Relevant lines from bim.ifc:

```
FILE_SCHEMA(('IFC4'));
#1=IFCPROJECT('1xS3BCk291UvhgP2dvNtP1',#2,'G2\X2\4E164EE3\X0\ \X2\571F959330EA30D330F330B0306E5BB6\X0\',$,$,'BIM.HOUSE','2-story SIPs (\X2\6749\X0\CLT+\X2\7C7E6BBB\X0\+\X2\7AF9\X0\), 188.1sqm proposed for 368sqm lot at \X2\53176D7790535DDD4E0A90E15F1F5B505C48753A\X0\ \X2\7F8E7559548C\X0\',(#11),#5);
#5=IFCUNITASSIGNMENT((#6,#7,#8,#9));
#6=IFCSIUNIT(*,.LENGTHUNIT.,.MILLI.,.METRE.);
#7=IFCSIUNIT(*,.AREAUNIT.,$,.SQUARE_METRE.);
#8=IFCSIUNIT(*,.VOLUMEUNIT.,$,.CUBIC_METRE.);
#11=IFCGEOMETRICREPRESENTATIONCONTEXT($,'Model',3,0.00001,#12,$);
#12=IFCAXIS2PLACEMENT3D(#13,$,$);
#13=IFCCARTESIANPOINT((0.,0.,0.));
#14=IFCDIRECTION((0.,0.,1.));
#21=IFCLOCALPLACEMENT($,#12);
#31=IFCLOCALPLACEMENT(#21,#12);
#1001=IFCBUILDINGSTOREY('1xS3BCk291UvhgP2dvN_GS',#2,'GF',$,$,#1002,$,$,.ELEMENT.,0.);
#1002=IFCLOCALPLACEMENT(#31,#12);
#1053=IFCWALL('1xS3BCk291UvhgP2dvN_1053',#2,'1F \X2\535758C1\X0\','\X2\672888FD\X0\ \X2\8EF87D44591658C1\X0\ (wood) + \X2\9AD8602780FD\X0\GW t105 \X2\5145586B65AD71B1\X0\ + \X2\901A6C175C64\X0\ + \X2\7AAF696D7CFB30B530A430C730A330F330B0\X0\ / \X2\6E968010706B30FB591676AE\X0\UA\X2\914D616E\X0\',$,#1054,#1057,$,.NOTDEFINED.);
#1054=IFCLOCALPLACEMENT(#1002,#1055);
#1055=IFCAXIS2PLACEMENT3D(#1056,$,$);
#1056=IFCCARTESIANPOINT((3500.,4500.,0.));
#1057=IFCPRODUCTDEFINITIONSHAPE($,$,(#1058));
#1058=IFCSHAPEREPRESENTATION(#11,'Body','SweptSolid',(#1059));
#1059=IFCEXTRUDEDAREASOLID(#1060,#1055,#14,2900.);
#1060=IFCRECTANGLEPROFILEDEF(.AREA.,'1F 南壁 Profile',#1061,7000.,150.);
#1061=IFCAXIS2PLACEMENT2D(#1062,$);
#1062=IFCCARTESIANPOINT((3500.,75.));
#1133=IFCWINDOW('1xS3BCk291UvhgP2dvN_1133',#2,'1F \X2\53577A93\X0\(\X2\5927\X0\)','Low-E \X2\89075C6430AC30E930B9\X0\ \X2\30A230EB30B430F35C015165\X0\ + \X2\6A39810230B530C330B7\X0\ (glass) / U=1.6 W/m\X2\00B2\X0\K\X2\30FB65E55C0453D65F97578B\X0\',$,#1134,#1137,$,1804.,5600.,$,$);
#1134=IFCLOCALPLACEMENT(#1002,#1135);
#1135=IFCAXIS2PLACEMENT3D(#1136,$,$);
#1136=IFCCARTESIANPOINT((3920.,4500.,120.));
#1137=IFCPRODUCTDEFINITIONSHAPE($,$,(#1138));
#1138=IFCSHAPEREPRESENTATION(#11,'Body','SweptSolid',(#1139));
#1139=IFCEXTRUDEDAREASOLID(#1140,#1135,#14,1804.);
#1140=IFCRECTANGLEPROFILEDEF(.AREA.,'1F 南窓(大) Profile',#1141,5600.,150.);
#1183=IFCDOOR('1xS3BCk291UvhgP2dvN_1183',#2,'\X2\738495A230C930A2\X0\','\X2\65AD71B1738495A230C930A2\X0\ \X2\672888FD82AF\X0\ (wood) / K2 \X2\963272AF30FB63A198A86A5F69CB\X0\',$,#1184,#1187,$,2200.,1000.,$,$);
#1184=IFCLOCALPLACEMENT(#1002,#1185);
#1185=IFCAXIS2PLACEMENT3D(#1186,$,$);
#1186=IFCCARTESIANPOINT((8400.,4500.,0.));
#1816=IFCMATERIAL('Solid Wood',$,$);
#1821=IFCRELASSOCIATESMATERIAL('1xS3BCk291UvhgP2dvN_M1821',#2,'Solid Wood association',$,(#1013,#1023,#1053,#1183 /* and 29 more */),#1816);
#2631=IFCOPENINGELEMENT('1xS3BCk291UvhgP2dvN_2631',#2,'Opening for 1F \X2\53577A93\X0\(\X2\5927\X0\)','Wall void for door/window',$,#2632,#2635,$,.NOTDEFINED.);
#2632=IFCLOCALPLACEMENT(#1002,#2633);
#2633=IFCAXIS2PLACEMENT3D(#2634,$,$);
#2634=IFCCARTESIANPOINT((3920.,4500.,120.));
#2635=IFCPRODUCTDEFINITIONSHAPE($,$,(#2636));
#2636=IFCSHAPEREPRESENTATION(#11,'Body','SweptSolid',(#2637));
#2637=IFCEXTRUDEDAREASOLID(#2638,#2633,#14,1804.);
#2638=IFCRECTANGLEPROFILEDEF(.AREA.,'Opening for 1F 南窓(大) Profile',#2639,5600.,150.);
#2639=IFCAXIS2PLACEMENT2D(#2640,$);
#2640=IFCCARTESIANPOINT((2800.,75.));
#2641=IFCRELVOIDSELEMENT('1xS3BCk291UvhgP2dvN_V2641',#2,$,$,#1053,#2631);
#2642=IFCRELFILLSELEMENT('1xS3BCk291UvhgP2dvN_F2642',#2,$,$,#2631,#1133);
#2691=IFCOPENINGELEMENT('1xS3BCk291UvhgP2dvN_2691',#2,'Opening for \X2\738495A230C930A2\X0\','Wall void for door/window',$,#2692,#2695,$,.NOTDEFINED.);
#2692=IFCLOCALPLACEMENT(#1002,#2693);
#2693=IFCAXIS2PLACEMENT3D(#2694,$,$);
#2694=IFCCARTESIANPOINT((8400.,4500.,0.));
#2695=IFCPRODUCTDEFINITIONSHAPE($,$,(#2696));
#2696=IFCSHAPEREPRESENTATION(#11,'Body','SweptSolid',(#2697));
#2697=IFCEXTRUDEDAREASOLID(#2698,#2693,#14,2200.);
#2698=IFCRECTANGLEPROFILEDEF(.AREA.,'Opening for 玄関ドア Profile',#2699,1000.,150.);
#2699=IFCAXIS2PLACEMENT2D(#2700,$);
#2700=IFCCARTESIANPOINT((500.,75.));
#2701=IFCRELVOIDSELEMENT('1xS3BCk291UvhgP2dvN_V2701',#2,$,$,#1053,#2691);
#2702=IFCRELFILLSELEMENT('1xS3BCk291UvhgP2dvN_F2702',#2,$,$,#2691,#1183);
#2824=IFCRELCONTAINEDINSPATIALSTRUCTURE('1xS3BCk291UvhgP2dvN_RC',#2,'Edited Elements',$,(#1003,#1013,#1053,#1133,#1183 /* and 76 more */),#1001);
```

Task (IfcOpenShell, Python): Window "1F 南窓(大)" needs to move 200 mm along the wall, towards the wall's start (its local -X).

```python
import ifcopenshell
import ifcopenshell.api.geometry
import ifcopenshell.util.placement
import ifcopenshell.util.unit

model = ifcopenshell.open("bim.ifc")
unit_scale = ifcopenshell.util.unit.calculate_unit_scale(model)

window = model.by_id(1133)
opening = window.FillsVoids[0].RelatingOpeningElement
wall = opening.VoidsElements[0].RelatingBuildingElement

wall_matrix = ifcopenshell.util.placement.get_local_placement(wall.ObjectPlacement)
shift = wall_matrix[:3, 0] * -0.2 / unit_scale
before = ifcopenshell.util.placement.get_local_placement(window.ObjectPlacement)[:3, 3].copy()

# The window is not placed relative to its opening, so move both.
for product in (opening, window):
    matrix = ifcopenshell.util.placement.get_local_placement(product.ObjectPlacement)
    matrix[:3, 3] += shift
    ifcopenshell.api.geometry.edit_object_placement(model, product=product, matrix=matrix, is_si=False)

after = ifcopenshell.util.placement.get_local_placement(window.ObjectPlacement)[:3, 3]
print("window moved by", (after - before).round(3) + 0.0)

model.write("bim_rev.ifc")
```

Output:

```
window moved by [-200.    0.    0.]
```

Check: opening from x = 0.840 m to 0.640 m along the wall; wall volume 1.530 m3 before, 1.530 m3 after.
